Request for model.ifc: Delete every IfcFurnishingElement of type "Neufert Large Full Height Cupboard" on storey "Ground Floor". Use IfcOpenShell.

First a look at what the model holds.

```python
import ifcopenshell
import ifcopenshell.util.element

model = ifcopenshell.open("model.ifc")
print(model.schema)
storey = next(s for s in model.by_type("IfcBuildingStorey") if s.Name == "Ground Floor")
furniture = [e for e in ifcopenshell.util.element.get_decomposition(storey) if e.is_a("IfcFurnishingElement")]
seen = {}
for e in furniture:
    element_type = ifcopenshell.util.element.get_type(e)
    name = element_type.Name if element_type not in (None, e) else None
    seen[name] = seen.get(name, 0) + 1
for name, count in sorted(seen.items(), key=str):
    print(count, "x", name)
```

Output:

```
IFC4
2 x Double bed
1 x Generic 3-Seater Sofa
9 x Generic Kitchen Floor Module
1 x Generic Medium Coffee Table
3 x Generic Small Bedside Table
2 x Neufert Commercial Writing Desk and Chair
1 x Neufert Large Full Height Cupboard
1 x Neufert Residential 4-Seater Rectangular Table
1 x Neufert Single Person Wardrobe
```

```python
import ifcopenshell
import ifcopenshell.api.root
import ifcopenshell.util.element

model = ifcopenshell.open("model.ifc")

storey = next(s for s in model.by_type("IfcBuildingStorey") if s.Name == "Ground Floor")
furniture = [e for e in ifcopenshell.util.element.get_decomposition(storey) if e.is_a("IfcFurnishingElement")]
targets = [e for e in furniture if (t := ifcopenshell.util.element.get_type(e)) not in (None, e) and t.Name == "Neufert Large Full Height Cupboard"]

for e in targets:
    ifcopenshell.api.root.remove_product(model, product=e)
print(len(targets), "removed")

model.write("model_v2.ifc")
```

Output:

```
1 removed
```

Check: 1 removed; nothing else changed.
